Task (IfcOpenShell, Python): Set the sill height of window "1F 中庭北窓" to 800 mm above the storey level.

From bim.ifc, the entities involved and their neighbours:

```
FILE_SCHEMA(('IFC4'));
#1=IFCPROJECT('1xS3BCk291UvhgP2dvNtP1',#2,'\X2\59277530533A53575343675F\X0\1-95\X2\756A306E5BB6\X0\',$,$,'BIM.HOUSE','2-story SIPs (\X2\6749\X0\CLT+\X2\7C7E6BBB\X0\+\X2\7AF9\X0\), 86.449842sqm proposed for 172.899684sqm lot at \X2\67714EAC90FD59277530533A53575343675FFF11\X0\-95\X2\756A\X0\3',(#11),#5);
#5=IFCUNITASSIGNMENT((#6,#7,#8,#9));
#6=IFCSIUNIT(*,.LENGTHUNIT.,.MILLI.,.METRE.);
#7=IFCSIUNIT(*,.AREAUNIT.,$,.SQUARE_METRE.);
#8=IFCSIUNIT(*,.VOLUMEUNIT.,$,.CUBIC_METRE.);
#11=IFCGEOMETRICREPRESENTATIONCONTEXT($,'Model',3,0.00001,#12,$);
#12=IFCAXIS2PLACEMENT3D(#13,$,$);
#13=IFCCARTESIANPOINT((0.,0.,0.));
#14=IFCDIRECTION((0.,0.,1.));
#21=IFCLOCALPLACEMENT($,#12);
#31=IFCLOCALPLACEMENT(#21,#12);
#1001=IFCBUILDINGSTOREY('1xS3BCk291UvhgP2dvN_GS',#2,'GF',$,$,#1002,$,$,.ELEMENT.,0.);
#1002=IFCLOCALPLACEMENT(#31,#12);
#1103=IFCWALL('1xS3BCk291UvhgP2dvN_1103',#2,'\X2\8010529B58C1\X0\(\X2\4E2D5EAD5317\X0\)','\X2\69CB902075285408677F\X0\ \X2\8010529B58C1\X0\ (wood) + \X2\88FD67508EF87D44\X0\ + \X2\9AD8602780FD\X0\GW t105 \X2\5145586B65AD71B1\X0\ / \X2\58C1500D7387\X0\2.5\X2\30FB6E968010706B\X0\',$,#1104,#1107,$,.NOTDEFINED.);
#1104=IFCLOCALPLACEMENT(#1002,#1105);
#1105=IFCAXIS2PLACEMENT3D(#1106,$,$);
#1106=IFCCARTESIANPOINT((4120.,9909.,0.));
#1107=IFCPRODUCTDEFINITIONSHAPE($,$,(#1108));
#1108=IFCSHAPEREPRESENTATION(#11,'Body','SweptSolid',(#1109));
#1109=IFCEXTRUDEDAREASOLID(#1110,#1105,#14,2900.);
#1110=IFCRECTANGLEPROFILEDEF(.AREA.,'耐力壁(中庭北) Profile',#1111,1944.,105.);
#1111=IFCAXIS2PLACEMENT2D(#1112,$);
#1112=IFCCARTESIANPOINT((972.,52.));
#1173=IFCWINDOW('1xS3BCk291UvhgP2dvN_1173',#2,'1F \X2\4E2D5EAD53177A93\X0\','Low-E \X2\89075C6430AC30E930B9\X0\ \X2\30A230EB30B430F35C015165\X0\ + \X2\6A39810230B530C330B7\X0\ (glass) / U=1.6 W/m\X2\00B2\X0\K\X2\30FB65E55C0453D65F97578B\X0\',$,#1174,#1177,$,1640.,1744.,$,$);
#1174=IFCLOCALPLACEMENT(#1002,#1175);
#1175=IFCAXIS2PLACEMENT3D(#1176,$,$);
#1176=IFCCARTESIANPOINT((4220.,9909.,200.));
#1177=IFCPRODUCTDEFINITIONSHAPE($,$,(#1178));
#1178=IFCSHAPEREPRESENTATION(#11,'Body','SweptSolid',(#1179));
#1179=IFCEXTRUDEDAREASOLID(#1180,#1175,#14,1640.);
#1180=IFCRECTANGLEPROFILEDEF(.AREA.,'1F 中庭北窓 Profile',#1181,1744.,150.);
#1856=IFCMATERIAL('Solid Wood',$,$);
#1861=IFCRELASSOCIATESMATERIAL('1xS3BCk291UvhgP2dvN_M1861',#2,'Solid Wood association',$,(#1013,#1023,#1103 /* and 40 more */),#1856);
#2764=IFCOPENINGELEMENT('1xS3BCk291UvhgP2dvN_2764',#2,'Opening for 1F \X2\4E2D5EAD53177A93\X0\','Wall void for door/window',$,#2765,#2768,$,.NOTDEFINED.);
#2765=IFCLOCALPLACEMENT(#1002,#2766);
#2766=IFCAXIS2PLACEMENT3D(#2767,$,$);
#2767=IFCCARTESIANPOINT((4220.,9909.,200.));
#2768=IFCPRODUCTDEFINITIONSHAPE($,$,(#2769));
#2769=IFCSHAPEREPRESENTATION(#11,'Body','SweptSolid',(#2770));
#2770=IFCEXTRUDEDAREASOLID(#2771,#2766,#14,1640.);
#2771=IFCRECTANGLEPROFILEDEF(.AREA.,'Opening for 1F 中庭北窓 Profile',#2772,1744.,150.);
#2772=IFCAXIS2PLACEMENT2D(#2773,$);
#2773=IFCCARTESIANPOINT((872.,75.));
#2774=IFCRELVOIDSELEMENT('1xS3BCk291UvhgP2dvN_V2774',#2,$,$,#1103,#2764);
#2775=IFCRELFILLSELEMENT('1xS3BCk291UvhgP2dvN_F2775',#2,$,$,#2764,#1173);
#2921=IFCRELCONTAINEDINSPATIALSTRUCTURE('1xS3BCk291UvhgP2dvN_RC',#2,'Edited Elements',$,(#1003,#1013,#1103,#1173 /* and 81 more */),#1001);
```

```python
import numpy as np
import ifcopenshell
import ifcopenshell.api.geometry
import ifcopenshell.geom
import ifcopenshell.util.element
import ifcopenshell.util.placement
import ifcopenshell.util.shape
import ifcopenshell.util.unit

model = ifcopenshell.open("bim.ifc")
unit_scale = ifcopenshell.util.unit.calculate_unit_scale(model)

window = model.by_guid("1xS3BCk291UvhgP2dvN_1173")
opening = window.FillsVoids[0].RelatingOpeningElement
storey = ifcopenshell.util.element.get_container(window, ifc_class="IfcBuildingStorey")
level = ifcopenshell.util.placement.get_local_placement(storey.ObjectPlacement)[2, 3]

# The opening's origin need not be at the sill, so measure its lowest point.
shape = ifcopenshell.geom.create_shape(ifcopenshell.geom.settings(), opening)
bottom = ifcopenshell.util.shape.get_shape_bottom_elevation(shape, shape.geometry) / unit_scale
dz = level + 800.0 - bottom

shift = np.array([0.0, 0.0, dz])
# The window is not placed relative to its opening, so move both.
for product in (opening, window):
    matrix = ifcopenshell.util.placement.get_local_placement(product.ObjectPlacement)
    matrix[:3, 3] += shift
    ifcopenshell.api.geometry.edit_object_placement(model, product=product, matrix=matrix, is_si=False)

print(f"moved by {dz * unit_scale:+.3f} m")

model.write("bim_updated.ifc")
```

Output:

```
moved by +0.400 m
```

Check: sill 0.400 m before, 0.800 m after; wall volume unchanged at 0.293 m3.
